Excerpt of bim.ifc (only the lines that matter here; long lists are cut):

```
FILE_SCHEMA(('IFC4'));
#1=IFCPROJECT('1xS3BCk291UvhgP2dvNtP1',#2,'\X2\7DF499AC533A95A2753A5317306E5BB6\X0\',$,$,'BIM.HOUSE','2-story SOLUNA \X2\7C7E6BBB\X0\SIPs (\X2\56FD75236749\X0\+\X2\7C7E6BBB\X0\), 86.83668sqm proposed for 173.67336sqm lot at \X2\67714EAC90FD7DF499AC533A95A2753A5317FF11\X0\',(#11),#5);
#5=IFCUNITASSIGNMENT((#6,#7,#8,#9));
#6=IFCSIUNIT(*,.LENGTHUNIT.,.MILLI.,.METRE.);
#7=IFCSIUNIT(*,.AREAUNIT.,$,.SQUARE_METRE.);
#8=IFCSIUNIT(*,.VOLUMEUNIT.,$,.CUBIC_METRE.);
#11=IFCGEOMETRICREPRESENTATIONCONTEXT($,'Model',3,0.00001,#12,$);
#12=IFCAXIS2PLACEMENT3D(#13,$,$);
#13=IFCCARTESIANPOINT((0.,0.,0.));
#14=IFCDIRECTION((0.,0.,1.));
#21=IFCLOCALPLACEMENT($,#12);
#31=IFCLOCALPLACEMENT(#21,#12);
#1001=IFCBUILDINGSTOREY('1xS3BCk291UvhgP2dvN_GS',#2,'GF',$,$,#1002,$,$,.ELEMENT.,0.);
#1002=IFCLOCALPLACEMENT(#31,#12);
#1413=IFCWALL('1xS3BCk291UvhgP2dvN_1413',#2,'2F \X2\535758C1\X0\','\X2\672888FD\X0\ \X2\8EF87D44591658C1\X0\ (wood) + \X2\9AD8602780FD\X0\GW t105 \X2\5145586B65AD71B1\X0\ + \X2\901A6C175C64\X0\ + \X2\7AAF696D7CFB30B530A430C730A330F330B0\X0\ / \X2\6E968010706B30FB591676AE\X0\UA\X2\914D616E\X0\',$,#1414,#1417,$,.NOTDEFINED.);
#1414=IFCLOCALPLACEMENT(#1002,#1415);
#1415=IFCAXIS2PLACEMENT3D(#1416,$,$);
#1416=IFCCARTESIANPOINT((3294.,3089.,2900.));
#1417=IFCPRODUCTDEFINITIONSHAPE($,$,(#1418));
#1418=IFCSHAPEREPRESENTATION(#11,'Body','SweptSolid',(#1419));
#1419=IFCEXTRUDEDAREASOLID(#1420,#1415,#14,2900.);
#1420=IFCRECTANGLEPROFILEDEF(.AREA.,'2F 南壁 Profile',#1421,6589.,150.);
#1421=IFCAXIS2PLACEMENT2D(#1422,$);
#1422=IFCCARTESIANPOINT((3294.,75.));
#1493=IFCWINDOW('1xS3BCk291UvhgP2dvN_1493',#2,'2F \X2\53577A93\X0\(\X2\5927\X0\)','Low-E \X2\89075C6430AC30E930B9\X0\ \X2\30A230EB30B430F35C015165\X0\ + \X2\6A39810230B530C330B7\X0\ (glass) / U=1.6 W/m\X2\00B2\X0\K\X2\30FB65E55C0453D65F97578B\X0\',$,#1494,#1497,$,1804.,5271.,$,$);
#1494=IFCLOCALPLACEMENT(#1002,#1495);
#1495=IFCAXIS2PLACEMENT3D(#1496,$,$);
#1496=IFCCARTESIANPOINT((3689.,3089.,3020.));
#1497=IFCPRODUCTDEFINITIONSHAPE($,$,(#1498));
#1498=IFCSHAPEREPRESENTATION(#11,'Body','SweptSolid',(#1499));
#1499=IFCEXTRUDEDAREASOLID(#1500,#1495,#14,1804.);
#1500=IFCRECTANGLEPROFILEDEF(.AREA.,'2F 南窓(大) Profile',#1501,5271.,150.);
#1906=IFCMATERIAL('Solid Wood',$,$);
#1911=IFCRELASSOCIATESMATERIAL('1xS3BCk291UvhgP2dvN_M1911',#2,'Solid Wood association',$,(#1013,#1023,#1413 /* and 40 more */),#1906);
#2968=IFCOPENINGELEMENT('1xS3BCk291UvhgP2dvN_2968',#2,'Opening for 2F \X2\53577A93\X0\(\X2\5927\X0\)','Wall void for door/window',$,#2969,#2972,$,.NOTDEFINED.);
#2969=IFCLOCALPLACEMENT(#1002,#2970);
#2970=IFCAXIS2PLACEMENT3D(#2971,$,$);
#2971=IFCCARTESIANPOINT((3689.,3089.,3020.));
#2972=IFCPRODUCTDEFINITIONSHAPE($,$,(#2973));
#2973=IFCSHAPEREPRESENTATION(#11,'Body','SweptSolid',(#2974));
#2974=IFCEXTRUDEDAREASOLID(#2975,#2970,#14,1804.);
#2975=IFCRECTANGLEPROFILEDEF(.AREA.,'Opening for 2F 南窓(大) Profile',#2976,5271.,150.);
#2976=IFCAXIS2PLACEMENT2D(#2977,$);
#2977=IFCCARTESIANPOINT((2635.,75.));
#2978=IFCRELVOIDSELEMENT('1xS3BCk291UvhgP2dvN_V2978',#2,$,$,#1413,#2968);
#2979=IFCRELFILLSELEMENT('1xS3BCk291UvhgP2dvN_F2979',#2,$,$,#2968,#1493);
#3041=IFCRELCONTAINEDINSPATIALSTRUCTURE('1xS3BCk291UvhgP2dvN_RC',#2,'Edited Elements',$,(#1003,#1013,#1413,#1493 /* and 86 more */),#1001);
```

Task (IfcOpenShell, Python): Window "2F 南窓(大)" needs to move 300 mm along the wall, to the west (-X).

```python
import ifcopenshell
import ifcopenshell.api.geometry
import ifcopenshell.util.placement

model = ifcopenshell.open("bim.ifc")

window = model.by_guid("1xS3BCk291UvhgP2dvN_1493")
opening = window.FillsVoids[0].RelatingOpeningElement
wall = opening.VoidsElements[0].RelatingBuildingElement

wall_matrix = ifcopenshell.util.placement.get_local_placement(wall.ObjectPlacement)
shift = wall_matrix[:3, 0] * -300.0
before = ifcopenshell.util.placement.get_local_placement(window.ObjectPlacement)[:3, 3].copy()

# The window is not placed relative to its opening, so move both.
for product in (opening, window):
    matrix = ifcopenshell.util.placement.get_local_placement(product.ObjectPlacement)
    matrix[:3, 3] += shift
    ifcopenshell.api.geometry.edit_object_placement(model, product=product, matrix=matrix, is_si=False)

after = ifcopenshell.util.placement.get_local_placement(window.ObjectPlacement)[:3, 3]
print("window moved by", (after - before).round(3) + 0.0)

model.write("bim_updated.ifc")
```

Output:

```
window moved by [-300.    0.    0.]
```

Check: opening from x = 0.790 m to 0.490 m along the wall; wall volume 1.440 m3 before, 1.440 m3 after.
